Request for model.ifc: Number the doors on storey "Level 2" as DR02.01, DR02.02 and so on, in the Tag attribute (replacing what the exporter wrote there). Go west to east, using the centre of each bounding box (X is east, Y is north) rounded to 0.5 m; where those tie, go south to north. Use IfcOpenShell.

First a look at what the model holds.

```python
import ifcopenshell
import ifcopenshell.util.element
import ifcopenshell.util.placement

model = ifcopenshell.open("model.ifc")
print(model.schema)
storey = next(s for s in model.by_type("IfcBuildingStorey") if s.Name == "Level 2")
doors = [e for e in ifcopenshell.util.element.get_decomposition(storey) if e.is_a("IfcDoor")]
for e in sorted(doors, key=lambda e: e.id()):
    origin = ifcopenshell.util.placement.get_local_placement(e.ObjectPlacement)[:3, 3]
    print(e.id(), e.Tag, e.Name, origin.round(2) + 0.0, sep=" | ")
```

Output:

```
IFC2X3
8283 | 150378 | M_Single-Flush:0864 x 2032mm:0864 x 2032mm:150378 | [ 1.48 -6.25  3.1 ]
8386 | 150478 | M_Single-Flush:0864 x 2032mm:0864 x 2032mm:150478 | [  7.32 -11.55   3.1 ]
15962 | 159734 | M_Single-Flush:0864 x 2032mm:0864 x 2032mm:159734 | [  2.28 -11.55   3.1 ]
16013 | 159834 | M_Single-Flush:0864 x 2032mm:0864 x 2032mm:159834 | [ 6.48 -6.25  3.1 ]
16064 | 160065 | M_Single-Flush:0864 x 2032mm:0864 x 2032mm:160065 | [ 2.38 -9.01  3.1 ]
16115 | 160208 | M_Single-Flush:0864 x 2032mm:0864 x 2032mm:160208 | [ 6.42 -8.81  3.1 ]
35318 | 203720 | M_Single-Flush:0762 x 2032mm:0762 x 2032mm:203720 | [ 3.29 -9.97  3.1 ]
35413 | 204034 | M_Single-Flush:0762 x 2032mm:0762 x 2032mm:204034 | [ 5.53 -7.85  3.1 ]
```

```python
import ifcopenshell
import ifcopenshell.geom
import ifcopenshell.util.element
import ifcopenshell.util.shape

model = ifcopenshell.open("model.ifc")
settings = ifcopenshell.geom.settings()
settings.set("use-world-coords", True)


def centre(element):
    shape = ifcopenshell.geom.create_shape(settings, element)
    return ifcopenshell.util.shape.get_bbox_centroid(shape.geometry)


storey = next(s for s in model.by_type("IfcBuildingStorey") if s.Name == "Level 2")
doors = [e for e in ifcopenshell.util.element.get_decomposition(storey) if e.is_a("IfcDoor")]

# Insertion points can sit at a corner or the storey origin, so sort by the geometry (in metres).
centres = {e: centre(e) for e in doors}
doors.sort(key=lambda e: (round(centres[e][0] / 0.5), centres[e][1]))

for i, e in enumerate(doors, start=1):
    number = f"DR02.{i:02d}"
    e.Tag = number
    print(e.id(), number)

model.write("model_v2.ifc")
```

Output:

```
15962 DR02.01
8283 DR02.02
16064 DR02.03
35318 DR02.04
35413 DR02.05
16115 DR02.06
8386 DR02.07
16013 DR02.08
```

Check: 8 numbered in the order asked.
